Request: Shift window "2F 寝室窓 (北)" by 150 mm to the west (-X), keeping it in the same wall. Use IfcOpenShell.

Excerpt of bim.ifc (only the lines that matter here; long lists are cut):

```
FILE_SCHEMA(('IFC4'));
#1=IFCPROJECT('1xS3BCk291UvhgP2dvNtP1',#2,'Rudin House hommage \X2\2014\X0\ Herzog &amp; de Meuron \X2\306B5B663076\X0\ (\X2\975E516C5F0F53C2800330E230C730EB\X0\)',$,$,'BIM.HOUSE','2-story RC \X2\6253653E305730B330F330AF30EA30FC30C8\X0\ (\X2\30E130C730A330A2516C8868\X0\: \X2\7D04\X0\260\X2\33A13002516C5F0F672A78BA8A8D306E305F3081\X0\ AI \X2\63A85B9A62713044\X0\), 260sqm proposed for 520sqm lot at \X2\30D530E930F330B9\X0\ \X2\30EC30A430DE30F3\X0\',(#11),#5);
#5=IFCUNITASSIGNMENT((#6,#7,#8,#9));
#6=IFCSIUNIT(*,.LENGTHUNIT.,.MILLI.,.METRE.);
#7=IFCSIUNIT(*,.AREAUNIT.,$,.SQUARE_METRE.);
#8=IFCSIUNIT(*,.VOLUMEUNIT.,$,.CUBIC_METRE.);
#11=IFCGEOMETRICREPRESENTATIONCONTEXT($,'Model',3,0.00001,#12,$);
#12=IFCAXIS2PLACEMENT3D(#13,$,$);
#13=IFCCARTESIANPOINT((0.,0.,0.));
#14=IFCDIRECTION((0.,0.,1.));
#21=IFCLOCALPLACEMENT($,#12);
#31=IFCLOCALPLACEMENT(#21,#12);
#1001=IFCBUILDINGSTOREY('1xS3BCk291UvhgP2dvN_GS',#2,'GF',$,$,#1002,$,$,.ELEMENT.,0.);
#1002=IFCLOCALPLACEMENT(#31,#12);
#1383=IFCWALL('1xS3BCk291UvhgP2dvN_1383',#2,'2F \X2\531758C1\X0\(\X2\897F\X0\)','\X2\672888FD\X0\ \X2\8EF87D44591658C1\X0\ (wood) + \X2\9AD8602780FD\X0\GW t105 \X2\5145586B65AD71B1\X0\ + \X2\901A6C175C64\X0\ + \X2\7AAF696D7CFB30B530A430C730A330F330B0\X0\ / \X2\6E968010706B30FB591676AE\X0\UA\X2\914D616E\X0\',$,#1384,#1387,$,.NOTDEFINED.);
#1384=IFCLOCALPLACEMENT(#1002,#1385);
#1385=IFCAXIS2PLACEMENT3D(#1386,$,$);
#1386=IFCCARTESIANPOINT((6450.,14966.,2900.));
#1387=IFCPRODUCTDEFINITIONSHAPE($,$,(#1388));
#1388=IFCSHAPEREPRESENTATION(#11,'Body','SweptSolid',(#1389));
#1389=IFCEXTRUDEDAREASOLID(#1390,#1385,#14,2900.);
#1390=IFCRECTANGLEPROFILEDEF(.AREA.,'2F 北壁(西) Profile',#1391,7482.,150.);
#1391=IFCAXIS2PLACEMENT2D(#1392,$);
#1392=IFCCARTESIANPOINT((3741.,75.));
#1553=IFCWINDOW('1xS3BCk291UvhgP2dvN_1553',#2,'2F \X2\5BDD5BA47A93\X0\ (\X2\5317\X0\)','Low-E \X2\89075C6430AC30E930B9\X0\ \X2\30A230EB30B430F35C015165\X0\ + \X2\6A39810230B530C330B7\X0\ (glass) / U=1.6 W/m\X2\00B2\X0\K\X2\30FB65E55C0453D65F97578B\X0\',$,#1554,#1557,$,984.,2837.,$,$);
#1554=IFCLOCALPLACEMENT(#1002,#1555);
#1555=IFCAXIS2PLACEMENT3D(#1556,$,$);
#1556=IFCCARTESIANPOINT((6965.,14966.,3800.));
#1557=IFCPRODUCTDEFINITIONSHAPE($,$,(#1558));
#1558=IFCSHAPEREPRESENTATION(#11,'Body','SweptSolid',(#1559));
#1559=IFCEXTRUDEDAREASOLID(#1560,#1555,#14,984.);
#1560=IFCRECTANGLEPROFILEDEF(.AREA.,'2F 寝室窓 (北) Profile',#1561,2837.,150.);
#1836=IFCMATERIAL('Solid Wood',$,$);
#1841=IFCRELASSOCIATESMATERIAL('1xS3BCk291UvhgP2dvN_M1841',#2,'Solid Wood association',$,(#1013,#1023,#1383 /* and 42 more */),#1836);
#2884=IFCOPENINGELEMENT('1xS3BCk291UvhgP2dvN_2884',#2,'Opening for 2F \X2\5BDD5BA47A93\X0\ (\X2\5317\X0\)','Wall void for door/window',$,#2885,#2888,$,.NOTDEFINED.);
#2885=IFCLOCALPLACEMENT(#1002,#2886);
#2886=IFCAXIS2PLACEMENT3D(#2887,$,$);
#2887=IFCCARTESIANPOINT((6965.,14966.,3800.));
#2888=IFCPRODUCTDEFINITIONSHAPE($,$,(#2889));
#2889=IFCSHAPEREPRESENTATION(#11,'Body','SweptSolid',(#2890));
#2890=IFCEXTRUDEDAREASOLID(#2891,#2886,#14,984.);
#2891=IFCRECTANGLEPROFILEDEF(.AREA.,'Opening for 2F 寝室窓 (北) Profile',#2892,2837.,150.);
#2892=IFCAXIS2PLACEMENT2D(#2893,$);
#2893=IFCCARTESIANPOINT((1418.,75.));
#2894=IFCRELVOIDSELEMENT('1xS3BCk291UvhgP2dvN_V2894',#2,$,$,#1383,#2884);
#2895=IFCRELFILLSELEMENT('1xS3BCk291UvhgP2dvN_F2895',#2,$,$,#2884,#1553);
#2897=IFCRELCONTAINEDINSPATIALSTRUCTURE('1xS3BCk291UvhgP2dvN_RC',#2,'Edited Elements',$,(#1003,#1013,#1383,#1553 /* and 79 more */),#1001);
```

```python
import ifcopenshell
import ifcopenshell.api.geometry
import ifcopenshell.util.placement

model = ifcopenshell.open("bim.ifc")

window = model.by_guid("1xS3BCk291UvhgP2dvN_1553")
opening = window.FillsVoids[0].RelatingOpeningElement
wall = opening.VoidsElements[0].RelatingBuildingElement

wall_matrix = ifcopenshell.util.placement.get_local_placement(wall.ObjectPlacement)
shift = wall_matrix[:3, 0] * -150.0
before = ifcopenshell.util.placement.get_local_placement(window.ObjectPlacement)[:3, 3].copy()

# The window is not placed relative to its opening, so move both.
for product in (opening, window):
    matrix = ifcopenshell.util.placement.get_local_placement(product.ObjectPlacement)
    matrix[:3, 3] += shift
    ifcopenshell.api.geometry.edit_object_placement(model, product=product, matrix=matrix, is_si=False)

after = ifcopenshell.util.placement.get_local_placement(window.ObjectPlacement)[:3, 3]
print("window moved by", (after - before).round(3) + 0.0)

model.write("bim_updated.ifc")
```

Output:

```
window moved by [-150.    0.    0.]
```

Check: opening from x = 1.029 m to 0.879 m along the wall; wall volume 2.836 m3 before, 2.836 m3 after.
